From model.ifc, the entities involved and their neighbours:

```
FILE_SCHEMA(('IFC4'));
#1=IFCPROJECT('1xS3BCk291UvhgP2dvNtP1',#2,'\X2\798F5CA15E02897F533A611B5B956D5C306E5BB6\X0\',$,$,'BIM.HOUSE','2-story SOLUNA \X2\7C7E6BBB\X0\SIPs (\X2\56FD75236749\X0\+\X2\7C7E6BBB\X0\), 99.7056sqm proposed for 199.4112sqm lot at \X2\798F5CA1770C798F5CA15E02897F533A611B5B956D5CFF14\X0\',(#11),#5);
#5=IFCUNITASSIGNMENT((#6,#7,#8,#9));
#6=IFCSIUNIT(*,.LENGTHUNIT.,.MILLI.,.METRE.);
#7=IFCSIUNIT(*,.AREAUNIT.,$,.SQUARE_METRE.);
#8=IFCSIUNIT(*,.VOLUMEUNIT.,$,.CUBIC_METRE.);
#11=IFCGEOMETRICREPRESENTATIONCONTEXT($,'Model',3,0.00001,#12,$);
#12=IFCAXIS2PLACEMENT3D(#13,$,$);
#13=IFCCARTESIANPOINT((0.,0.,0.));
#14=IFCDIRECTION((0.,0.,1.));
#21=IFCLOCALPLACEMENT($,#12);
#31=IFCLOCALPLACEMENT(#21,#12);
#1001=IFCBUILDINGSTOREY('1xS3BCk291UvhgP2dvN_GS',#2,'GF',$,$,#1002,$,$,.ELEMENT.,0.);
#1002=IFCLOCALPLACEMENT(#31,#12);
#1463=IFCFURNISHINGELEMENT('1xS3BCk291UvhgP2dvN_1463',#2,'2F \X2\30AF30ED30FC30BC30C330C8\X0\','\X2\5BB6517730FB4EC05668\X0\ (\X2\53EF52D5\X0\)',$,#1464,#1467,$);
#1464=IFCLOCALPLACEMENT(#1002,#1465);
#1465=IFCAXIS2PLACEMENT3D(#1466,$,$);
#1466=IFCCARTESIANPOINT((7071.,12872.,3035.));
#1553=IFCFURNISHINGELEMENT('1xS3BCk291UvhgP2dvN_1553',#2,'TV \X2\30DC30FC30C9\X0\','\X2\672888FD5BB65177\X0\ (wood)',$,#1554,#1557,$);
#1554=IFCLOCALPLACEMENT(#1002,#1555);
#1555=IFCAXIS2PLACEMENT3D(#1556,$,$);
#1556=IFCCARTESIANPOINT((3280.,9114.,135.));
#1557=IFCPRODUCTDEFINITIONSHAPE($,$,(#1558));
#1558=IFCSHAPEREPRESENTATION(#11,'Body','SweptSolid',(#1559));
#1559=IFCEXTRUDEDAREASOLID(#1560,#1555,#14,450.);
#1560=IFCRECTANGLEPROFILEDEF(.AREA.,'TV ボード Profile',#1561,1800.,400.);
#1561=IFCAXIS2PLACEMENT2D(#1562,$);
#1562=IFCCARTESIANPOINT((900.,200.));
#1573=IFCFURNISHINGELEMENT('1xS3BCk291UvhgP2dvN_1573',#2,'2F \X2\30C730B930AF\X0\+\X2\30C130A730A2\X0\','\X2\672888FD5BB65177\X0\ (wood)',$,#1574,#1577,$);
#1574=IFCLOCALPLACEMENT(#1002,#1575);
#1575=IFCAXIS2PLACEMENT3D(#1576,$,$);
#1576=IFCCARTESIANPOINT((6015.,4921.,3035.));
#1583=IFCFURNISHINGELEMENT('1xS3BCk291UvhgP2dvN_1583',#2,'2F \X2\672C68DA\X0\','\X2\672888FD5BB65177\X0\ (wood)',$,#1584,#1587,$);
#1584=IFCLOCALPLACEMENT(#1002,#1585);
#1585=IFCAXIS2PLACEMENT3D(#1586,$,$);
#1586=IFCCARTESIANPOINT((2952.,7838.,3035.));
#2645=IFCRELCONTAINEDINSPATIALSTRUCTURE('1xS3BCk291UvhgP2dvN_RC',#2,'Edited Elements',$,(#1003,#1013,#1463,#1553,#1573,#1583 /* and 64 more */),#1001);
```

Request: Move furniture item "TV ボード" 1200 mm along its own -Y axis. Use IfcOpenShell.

```python
import ifcopenshell
import ifcopenshell.api.geometry
import ifcopenshell.util.placement

model = ifcopenshell.open("model.ifc")

item = model.by_guid("1xS3BCk291UvhgP2dvN_1553")
matrix = ifcopenshell.util.placement.get_local_placement(item.ObjectPlacement)
matrix[:3, 3] -= matrix[:3, 1] * 1200.0
ifcopenshell.api.geometry.edit_object_placement(model, product=item, matrix=matrix, is_si=False)

print(ifcopenshell.util.placement.get_local_placement(item.ObjectPlacement).round(3) + 0.0)

model.write("model_rev.ifc")
```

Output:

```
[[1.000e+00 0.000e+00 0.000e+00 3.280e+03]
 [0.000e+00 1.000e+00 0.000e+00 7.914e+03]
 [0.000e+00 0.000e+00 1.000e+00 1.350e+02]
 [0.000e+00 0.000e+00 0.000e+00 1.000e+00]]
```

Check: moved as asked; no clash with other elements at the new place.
